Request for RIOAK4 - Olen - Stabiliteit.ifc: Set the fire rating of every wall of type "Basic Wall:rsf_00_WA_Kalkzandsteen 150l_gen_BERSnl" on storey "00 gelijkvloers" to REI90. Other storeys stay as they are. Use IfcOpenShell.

First a look at what the model holds.

```python
import ifcopenshell
import ifcopenshell.util.element

model = ifcopenshell.open("RIOAK4 - Olen - Stabiliteit.ifc")
print(model.schema)
storey = next(s for s in model.by_type("IfcBuildingStorey") if s.Name == "00 gelijkvloers")
walls = [e for e in ifcopenshell.util.element.get_decomposition(storey) if e.is_a("IfcWall")]
seen = {}
for e in walls:
    element_type = ifcopenshell.util.element.get_type(e)
    key = (element_type.Name if element_type != e and element_type else None, ifcopenshell.util.element.get_pset(e, "Pset_WallCommon", "FireRating"))
    seen[key] = seen.get(key, 0) + 1
for (name, value), count in sorted(seen.items(), key=str):
    print(count, "x", name, "|", value)
```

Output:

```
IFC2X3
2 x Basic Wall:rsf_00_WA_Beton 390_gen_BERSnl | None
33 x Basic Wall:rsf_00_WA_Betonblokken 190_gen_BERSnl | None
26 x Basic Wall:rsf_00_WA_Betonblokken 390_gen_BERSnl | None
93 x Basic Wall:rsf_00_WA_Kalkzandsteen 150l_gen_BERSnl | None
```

```python
import ifcopenshell
import ifcopenshell.api.pset
import ifcopenshell.util.element

model = ifcopenshell.open("RIOAK4 - Olen - Stabiliteit.ifc")

storey = next(s for s in model.by_type("IfcBuildingStorey") if s.Name == "00 gelijkvloers")
walls = [e for e in ifcopenshell.util.element.get_decomposition(storey) if e.is_a("IfcWall")]

count = 0
for e in walls:
    element_type = ifcopenshell.util.element.get_type(e)
    if element_type in (None, e) or element_type.Name != "Basic Wall:rsf_00_WA_Kalkzandsteen 150l_gen_BERSnl":
        continue
    # add_pset returns the element's existing set when there is one.
    pset = ifcopenshell.api.pset.add_pset(model, product=e, name="Pset_WallCommon")
    ifcopenshell.api.pset.edit_pset(model, pset=pset, properties={"FireRating": "REI90"})
    count += 1

print(count, "walls updated")

model.write("RIOAK4 - Olen - Stabiliteit_v2.ifc")
```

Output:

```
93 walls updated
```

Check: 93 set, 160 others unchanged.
